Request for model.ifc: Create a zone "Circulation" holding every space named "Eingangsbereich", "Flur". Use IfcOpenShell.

First a look at what the model holds.

```python
import ifcopenshell

model = ifcopenshell.open("model.ifc")
print(model.schema)
seen = {}
for space in model.by_type("IfcSpace"):
    seen[space.LongName] = seen.get(space.LongName, 0) + 1
for name, count in sorted(seen.items(), key=str):
    print(count, "x", name)
print("zones:", [z.Name for z in model.by_type("IfcZone")][:20])
```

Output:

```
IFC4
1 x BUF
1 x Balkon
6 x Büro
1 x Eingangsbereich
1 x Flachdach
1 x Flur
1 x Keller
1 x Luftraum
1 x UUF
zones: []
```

```python
import ifcopenshell
import ifcopenshell.api.group
import ifcopenshell.api.root

model = ifcopenshell.open("model.ifc")

names = {"Eingangsbereich", "Flur"}
spaces = [s for s in model.by_type("IfcSpace") if s.LongName in names]

zone = ifcopenshell.api.root.create_entity(model, ifc_class="IfcZone", name="Circulation")
ifcopenshell.api.group.assign_group(model, products=spaces, group=zone)
print(len(spaces), "spaces in", zone.Name)

model.write("model_edited.ifc")
```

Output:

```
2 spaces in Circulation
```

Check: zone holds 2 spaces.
